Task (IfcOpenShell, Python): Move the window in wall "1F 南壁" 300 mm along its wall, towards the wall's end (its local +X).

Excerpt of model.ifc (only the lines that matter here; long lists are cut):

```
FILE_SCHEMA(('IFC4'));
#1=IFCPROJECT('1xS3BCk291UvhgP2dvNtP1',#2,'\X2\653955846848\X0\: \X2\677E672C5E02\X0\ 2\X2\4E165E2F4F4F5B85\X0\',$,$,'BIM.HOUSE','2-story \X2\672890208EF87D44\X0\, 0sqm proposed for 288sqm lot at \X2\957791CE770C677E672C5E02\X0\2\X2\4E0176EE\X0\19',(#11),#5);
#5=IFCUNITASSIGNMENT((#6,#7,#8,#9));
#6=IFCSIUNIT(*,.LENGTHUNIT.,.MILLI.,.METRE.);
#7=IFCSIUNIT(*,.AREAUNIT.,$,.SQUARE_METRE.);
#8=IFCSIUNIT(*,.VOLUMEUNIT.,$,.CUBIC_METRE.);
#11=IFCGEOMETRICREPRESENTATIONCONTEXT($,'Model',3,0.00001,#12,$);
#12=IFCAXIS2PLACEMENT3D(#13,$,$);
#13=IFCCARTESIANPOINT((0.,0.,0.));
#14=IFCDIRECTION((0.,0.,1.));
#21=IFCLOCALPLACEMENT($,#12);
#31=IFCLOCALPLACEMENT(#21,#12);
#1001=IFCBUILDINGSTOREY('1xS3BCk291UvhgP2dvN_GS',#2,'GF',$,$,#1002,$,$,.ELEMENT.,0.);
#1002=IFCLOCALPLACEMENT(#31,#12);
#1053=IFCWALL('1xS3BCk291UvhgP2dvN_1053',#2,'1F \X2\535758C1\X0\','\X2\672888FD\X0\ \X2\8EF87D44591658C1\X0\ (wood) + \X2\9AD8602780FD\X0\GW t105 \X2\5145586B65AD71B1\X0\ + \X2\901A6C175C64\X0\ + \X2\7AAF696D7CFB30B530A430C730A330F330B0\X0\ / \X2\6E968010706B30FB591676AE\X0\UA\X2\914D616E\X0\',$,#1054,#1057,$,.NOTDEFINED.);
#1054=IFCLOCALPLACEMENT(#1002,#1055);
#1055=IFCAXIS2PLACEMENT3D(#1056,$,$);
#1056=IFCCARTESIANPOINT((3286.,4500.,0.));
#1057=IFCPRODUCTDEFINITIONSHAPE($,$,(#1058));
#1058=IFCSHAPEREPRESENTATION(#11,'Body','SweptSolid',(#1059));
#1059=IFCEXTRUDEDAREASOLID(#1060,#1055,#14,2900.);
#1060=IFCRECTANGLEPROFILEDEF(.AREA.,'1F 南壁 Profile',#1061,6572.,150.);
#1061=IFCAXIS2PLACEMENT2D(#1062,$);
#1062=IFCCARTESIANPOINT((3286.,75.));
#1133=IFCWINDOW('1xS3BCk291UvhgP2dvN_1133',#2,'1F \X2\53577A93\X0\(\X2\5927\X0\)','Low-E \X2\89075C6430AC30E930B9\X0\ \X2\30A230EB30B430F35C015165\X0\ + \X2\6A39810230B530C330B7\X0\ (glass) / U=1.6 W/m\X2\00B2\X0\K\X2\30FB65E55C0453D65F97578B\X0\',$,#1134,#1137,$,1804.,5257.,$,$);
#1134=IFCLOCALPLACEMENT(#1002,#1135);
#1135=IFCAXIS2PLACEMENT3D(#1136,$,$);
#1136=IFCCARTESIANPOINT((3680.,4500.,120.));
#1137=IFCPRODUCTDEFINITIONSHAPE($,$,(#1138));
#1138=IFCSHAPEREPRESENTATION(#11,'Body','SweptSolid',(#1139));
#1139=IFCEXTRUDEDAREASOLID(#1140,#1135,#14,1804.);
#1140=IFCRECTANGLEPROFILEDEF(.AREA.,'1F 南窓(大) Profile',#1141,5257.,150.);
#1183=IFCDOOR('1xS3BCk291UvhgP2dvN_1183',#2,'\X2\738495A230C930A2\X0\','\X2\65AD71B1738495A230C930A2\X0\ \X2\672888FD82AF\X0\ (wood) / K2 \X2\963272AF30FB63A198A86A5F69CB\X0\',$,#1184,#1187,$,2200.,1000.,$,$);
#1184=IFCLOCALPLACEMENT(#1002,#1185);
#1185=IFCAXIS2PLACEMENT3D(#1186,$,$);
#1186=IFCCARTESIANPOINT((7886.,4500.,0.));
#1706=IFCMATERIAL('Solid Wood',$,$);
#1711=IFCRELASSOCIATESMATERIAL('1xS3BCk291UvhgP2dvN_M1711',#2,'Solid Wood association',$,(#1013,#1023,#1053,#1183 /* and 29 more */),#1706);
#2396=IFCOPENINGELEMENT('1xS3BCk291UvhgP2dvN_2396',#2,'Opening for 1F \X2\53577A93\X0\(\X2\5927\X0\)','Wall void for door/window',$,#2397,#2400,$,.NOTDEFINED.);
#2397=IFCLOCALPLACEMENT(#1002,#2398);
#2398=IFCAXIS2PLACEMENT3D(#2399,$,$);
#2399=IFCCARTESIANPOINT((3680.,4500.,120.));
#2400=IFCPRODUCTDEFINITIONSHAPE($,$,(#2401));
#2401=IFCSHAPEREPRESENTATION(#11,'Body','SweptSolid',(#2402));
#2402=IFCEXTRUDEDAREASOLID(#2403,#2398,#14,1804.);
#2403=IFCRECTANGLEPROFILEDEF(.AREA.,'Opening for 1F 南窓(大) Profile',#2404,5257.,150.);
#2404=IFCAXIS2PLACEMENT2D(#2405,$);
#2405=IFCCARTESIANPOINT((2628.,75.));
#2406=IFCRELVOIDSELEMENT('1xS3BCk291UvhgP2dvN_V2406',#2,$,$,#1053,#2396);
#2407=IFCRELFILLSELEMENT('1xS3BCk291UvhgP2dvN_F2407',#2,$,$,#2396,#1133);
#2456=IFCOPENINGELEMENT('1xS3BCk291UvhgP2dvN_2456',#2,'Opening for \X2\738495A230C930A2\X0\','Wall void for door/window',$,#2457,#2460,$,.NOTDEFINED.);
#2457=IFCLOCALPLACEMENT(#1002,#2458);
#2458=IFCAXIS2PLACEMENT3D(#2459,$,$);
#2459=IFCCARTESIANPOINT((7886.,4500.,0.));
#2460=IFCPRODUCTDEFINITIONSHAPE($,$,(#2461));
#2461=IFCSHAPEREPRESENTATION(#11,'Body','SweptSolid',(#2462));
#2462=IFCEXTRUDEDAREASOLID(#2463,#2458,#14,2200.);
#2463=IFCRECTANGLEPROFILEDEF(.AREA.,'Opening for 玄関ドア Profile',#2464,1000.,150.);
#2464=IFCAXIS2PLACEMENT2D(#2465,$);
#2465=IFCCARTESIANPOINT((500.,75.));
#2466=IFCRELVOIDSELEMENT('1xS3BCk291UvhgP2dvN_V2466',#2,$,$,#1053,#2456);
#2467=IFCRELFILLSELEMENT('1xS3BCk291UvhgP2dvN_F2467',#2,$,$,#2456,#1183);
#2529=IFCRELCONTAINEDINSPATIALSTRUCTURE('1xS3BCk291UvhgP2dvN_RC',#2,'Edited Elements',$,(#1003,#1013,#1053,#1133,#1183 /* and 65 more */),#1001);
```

```python
import ifcopenshell
import ifcopenshell.api.geometry
import ifcopenshell.util.placement
import ifcopenshell.util.unit

model = ifcopenshell.open("model.ifc")
unit_scale = ifcopenshell.util.unit.calculate_unit_scale(model)

window = model.by_guid("1xS3BCk291UvhgP2dvN_1133")
opening = window.FillsVoids[0].RelatingOpeningElement
wall = opening.VoidsElements[0].RelatingBuildingElement

wall_matrix = ifcopenshell.util.placement.get_local_placement(wall.ObjectPlacement)
shift = wall_matrix[:3, 0] * 0.3 / unit_scale
before = ifcopenshell.util.placement.get_local_placement(window.ObjectPlacement)[:3, 3].copy()

# The window is not placed relative to its opening, so move both.
for product in (opening, window):
    matrix = ifcopenshell.util.placement.get_local_placement(product.ObjectPlacement)
    matrix[:3, 3] += shift
    ifcopenshell.api.geometry.edit_object_placement(model, product=product, matrix=matrix, is_si=False)

after = ifcopenshell.util.placement.get_local_placement(window.ObjectPlacement)[:3, 3]
print("window moved by", (after - before).round(3) + 0.0)

model.write("model-out.ifc")
```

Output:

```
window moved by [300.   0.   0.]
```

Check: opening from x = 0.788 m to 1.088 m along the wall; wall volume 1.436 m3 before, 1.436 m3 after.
